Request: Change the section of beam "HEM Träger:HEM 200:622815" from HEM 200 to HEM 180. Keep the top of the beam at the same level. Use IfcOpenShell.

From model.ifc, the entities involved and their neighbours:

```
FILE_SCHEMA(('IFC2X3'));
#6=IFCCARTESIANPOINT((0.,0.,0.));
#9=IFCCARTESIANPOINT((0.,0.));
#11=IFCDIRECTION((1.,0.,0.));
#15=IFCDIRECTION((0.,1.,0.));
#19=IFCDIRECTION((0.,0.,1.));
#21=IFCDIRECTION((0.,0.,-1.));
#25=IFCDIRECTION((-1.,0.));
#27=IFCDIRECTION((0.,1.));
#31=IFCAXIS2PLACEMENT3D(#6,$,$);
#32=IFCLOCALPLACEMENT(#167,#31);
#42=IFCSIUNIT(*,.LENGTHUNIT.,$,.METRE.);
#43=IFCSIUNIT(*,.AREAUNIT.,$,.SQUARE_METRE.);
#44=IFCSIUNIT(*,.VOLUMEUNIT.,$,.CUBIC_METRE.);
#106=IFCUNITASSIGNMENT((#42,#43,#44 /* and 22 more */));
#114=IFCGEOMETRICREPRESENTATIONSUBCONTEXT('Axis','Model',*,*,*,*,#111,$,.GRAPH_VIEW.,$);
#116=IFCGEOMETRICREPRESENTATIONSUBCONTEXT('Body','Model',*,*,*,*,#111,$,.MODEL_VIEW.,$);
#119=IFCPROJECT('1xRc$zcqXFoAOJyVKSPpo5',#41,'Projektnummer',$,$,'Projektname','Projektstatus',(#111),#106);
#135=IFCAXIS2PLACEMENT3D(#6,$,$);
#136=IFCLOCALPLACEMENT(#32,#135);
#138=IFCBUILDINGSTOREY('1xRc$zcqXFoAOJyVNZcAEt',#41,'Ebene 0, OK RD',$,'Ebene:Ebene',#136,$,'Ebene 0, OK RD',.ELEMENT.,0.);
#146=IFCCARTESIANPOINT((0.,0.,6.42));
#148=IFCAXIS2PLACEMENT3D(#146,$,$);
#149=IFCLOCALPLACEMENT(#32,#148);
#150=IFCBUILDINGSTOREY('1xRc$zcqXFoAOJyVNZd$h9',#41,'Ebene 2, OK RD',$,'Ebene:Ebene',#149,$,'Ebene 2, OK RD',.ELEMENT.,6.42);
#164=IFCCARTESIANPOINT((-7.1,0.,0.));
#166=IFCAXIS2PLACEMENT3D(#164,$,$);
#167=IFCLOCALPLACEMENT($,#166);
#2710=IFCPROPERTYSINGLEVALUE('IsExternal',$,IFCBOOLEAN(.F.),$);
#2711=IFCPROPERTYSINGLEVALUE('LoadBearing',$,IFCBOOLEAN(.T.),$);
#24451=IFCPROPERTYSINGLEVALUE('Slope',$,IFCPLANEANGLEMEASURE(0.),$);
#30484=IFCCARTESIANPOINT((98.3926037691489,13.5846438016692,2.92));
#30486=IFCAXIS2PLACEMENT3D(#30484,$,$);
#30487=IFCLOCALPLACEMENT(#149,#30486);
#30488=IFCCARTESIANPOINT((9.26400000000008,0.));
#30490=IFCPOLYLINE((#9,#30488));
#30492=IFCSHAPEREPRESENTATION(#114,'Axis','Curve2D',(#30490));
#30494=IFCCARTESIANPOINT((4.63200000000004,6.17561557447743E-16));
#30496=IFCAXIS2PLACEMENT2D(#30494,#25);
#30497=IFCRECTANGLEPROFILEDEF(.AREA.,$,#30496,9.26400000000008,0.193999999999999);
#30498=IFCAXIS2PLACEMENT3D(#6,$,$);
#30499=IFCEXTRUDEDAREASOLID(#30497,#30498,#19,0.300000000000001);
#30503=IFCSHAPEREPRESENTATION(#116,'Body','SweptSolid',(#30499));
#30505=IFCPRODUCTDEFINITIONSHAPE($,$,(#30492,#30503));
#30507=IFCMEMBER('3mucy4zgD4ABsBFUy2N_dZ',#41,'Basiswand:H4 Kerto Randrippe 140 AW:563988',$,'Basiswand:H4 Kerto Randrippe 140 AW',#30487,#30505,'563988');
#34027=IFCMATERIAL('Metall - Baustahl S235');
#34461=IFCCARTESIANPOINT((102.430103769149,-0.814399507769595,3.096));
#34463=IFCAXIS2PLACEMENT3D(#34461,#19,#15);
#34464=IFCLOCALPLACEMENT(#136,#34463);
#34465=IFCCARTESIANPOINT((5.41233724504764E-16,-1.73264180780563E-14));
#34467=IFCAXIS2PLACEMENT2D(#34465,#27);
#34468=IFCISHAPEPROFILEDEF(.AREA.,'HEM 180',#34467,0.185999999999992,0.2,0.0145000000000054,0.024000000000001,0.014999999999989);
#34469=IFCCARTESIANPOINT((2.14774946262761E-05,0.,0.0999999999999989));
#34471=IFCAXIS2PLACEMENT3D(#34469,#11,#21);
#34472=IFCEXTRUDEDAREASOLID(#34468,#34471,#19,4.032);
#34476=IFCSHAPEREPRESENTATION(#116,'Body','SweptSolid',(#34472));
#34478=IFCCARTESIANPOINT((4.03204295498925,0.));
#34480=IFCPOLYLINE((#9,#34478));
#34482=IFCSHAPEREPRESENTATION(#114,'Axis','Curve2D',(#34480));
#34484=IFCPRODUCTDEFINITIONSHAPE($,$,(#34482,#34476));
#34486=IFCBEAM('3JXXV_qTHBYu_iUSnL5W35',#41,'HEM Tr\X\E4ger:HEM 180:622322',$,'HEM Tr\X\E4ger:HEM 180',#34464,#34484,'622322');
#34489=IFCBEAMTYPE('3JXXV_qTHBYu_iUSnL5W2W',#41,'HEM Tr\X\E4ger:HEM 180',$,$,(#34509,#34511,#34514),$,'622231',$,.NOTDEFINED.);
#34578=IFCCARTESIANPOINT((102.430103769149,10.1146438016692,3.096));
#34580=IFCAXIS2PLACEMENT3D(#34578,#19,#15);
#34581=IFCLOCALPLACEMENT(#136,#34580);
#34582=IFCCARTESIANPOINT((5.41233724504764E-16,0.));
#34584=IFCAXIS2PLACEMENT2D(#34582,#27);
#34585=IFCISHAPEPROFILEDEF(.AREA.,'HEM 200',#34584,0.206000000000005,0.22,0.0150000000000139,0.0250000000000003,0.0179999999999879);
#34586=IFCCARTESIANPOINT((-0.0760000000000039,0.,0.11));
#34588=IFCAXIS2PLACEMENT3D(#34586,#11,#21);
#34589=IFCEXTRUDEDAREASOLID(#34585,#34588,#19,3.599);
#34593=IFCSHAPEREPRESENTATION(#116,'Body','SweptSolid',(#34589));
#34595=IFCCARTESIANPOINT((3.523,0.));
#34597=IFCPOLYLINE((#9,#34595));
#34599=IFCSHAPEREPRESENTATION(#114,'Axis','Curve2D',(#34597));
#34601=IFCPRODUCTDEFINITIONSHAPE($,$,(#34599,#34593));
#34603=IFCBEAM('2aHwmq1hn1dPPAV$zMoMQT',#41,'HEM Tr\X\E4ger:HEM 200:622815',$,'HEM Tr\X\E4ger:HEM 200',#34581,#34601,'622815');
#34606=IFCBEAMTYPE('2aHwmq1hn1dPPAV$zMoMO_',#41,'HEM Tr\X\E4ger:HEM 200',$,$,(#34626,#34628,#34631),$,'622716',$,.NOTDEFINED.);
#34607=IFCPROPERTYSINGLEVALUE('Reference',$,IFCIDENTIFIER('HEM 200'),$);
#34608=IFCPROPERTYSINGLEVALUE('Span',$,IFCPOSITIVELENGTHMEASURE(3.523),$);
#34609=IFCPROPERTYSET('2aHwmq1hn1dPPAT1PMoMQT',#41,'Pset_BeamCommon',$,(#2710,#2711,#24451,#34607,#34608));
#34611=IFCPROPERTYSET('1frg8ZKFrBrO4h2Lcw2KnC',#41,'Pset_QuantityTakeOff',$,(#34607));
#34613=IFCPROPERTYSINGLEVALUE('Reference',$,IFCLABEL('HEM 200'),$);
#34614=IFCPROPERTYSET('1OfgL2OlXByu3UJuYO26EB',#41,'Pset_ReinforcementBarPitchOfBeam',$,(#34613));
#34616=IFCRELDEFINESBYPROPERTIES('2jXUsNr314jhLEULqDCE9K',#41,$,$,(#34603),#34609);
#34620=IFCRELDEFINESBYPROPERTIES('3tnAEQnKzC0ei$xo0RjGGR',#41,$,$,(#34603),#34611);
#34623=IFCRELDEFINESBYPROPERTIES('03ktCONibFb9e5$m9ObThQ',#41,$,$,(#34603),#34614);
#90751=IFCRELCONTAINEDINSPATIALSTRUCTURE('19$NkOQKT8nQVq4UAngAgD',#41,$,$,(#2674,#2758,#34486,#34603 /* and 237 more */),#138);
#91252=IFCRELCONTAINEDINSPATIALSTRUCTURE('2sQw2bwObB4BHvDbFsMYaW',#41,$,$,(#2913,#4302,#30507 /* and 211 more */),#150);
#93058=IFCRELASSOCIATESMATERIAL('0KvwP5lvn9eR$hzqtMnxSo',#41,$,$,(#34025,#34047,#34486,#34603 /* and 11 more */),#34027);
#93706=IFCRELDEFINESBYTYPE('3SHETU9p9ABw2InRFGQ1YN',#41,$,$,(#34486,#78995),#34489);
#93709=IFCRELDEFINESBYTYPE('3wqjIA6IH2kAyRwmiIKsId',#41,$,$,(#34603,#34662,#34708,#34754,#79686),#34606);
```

```python
import ifcopenshell
import ifcopenshell.api.pset
import ifcopenshell.api.type
import ifcopenshell.util.element
import ifcopenshell.util.representation

model = ifcopenshell.open("model.ifc")

member = model.by_id(34603)
source = next(p for p in model.by_type("IfcIShapeProfileDef") if p.ProfileName == "HEM 180")

body = ifcopenshell.util.representation.get_representation(member, "Model", "Body")
solid = body.Items[0]
old_profile = solid.SweptArea

# Copy the section's sizes but keep this member's own profile position.
profile = ifcopenshell.util.element.copy(model, source)
# Profiles are centred, so shift by half the change in depth to hold the top.
shift = (old_profile.OverallDepth - profile.OverallDepth) / 2
x, y = old_profile.Position.Location.Coordinates
up = (-1.0, 0.0)  # upwards, in the solid's own plane
location = model.createIfcCartesianPoint((x + up[0] * shift, y + up[1] * shift))
profile.Position = model.createIfcAxis2Placement2D(location, old_profile.Position.RefDirection)
solid.SweptArea = profile
if not model.get_total_inverses(old_profile):
    ifcopenshell.util.element.remove_deep2(model, old_profile)

new_type = model.by_guid("3JXXV_qTHBYu_iUSnL5W2W")
ifcopenshell.api.type.assign_type(
    model, related_objects=[member], relating_type=new_type, should_map_representations=False
)
member.Name = member.Name.replace("HEM 200", "HEM 180")
member.ObjectType = "HEM Träger:HEM 180"
pset = model.by_id(ifcopenshell.util.element.get_pset(member, "Pset_BeamCommon", should_inherit=False)["id"])
ifcopenshell.api.pset.edit_pset(model, pset=pset, properties={"Reference": "HEM 180"})
pset = model.by_id(ifcopenshell.util.element.get_pset(member, "Pset_QuantityTakeOff", should_inherit=False)["id"])
ifcopenshell.api.pset.edit_pset(model, pset=pset, properties={"Reference": "HEM 180"})
pset = model.by_id(ifcopenshell.util.element.get_pset(member, "Pset_ReinforcementBarPitchOfBeam", should_inherit=False)["id"])
ifcopenshell.api.pset.edit_pset(model, pset=pset, properties={"Reference": "HEM 180"})

print(solid.SweptArea)

model.write("model_edited.ifc")
```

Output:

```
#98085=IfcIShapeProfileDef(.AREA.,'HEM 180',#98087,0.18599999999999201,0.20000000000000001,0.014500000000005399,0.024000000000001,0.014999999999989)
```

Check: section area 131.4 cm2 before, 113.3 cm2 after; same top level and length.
